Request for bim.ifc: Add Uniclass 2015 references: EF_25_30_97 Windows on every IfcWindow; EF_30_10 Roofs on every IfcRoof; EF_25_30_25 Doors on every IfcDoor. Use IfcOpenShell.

First a look at what the model holds.

```python
import ifcopenshell

model = ifcopenshell.open("bim.ifc")
print(model.schema)
print("classifications:", [c.Name for c in model.by_type("IfcClassification")])
for ifc_class in ("IfcDoor", "IfcRoof", "IfcStair", "IfcWall", "IfcWindow"):
    print(ifc_class, len(model.by_type(ifc_class)))
```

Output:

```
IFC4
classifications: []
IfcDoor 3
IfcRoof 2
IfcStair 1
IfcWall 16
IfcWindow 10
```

```python
import ifcopenshell
import ifcopenshell.api.classification

model = ifcopenshell.open("bim.ifc")

system = ifcopenshell.api.classification.add_classification(model, classification="Uniclass 2015")

codes = {
    "IfcWindow": ("EF_25_30_97", "Windows"),
    "IfcRoof": ("EF_30_10", "Roofs"),
    "IfcDoor": ("EF_25_30_25", "Doors"),
}
for ifc_class, (code, name) in codes.items():
    products = model.by_type(ifc_class)
    ifcopenshell.api.classification.add_reference(
        model, products=products, classification=system, identification=code, name=name
    )
    print(code, len(products))

model.write("bim_rev.ifc")
```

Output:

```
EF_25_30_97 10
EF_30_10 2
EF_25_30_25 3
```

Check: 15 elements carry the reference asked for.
